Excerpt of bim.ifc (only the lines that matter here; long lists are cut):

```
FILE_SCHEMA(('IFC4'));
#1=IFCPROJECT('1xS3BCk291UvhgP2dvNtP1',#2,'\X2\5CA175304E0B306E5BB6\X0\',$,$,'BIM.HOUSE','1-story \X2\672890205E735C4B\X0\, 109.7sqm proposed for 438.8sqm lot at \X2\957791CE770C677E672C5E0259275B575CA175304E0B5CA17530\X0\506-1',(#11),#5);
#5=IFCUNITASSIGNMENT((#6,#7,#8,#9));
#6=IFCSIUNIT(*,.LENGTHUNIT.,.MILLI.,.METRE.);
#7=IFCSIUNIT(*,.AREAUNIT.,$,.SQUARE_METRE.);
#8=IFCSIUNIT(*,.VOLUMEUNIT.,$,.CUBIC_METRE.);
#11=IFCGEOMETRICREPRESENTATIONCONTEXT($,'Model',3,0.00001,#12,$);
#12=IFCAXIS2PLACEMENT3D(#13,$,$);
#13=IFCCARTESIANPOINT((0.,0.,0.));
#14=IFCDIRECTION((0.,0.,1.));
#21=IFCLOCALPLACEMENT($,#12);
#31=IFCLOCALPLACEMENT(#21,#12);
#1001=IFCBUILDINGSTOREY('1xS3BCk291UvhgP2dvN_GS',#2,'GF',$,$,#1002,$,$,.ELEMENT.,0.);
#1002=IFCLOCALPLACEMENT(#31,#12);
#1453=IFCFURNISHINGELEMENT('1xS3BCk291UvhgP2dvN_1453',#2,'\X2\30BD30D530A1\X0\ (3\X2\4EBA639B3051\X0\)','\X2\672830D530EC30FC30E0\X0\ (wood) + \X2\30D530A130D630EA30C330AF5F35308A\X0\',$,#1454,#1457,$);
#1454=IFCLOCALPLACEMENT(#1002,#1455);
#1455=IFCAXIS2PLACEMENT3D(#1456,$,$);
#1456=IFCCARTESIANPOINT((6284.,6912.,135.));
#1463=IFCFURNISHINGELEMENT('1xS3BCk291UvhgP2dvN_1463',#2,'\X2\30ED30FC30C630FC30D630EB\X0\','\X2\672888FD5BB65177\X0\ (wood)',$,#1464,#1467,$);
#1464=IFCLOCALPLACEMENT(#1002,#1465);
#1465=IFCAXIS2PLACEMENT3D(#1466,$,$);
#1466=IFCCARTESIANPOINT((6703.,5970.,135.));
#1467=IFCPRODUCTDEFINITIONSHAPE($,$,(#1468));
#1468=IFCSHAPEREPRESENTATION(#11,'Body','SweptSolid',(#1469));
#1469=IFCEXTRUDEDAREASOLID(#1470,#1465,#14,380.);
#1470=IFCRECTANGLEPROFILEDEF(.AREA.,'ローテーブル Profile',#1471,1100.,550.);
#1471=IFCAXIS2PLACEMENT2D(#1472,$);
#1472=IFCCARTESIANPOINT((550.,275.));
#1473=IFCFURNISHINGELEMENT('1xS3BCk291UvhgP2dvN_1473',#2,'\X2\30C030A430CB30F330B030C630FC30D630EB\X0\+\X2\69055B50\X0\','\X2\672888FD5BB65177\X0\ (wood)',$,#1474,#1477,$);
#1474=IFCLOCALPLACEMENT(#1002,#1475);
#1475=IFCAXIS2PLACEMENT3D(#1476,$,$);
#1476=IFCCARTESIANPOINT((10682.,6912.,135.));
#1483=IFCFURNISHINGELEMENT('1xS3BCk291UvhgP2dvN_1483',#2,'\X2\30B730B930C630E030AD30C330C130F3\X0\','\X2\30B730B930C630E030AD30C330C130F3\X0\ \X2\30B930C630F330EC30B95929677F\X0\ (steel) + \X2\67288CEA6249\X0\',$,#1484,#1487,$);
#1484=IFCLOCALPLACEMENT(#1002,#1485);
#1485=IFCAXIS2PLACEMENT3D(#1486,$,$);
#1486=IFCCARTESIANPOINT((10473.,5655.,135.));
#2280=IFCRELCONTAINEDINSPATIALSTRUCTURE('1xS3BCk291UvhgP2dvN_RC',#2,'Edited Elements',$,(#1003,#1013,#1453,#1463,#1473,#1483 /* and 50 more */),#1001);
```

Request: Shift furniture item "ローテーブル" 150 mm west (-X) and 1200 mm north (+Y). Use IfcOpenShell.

```python
import ifcopenshell
import ifcopenshell.api.geometry
import ifcopenshell.util.placement

model = ifcopenshell.open("bim.ifc")

item = model.by_guid("1xS3BCk291UvhgP2dvN_1463")
matrix = ifcopenshell.util.placement.get_local_placement(item.ObjectPlacement)
matrix[0, 3] -= 150.0
matrix[1, 3] += 1200.0
ifcopenshell.api.geometry.edit_object_placement(model, product=item, matrix=matrix, is_si=False)

print(ifcopenshell.util.placement.get_local_placement(item.ObjectPlacement).round(3) + 0.0)

model.write("bim_v2.ifc")
```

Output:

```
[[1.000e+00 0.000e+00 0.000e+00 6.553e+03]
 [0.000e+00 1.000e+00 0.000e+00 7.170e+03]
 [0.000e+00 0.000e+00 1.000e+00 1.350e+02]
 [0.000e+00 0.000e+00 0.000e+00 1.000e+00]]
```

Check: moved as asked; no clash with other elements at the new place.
